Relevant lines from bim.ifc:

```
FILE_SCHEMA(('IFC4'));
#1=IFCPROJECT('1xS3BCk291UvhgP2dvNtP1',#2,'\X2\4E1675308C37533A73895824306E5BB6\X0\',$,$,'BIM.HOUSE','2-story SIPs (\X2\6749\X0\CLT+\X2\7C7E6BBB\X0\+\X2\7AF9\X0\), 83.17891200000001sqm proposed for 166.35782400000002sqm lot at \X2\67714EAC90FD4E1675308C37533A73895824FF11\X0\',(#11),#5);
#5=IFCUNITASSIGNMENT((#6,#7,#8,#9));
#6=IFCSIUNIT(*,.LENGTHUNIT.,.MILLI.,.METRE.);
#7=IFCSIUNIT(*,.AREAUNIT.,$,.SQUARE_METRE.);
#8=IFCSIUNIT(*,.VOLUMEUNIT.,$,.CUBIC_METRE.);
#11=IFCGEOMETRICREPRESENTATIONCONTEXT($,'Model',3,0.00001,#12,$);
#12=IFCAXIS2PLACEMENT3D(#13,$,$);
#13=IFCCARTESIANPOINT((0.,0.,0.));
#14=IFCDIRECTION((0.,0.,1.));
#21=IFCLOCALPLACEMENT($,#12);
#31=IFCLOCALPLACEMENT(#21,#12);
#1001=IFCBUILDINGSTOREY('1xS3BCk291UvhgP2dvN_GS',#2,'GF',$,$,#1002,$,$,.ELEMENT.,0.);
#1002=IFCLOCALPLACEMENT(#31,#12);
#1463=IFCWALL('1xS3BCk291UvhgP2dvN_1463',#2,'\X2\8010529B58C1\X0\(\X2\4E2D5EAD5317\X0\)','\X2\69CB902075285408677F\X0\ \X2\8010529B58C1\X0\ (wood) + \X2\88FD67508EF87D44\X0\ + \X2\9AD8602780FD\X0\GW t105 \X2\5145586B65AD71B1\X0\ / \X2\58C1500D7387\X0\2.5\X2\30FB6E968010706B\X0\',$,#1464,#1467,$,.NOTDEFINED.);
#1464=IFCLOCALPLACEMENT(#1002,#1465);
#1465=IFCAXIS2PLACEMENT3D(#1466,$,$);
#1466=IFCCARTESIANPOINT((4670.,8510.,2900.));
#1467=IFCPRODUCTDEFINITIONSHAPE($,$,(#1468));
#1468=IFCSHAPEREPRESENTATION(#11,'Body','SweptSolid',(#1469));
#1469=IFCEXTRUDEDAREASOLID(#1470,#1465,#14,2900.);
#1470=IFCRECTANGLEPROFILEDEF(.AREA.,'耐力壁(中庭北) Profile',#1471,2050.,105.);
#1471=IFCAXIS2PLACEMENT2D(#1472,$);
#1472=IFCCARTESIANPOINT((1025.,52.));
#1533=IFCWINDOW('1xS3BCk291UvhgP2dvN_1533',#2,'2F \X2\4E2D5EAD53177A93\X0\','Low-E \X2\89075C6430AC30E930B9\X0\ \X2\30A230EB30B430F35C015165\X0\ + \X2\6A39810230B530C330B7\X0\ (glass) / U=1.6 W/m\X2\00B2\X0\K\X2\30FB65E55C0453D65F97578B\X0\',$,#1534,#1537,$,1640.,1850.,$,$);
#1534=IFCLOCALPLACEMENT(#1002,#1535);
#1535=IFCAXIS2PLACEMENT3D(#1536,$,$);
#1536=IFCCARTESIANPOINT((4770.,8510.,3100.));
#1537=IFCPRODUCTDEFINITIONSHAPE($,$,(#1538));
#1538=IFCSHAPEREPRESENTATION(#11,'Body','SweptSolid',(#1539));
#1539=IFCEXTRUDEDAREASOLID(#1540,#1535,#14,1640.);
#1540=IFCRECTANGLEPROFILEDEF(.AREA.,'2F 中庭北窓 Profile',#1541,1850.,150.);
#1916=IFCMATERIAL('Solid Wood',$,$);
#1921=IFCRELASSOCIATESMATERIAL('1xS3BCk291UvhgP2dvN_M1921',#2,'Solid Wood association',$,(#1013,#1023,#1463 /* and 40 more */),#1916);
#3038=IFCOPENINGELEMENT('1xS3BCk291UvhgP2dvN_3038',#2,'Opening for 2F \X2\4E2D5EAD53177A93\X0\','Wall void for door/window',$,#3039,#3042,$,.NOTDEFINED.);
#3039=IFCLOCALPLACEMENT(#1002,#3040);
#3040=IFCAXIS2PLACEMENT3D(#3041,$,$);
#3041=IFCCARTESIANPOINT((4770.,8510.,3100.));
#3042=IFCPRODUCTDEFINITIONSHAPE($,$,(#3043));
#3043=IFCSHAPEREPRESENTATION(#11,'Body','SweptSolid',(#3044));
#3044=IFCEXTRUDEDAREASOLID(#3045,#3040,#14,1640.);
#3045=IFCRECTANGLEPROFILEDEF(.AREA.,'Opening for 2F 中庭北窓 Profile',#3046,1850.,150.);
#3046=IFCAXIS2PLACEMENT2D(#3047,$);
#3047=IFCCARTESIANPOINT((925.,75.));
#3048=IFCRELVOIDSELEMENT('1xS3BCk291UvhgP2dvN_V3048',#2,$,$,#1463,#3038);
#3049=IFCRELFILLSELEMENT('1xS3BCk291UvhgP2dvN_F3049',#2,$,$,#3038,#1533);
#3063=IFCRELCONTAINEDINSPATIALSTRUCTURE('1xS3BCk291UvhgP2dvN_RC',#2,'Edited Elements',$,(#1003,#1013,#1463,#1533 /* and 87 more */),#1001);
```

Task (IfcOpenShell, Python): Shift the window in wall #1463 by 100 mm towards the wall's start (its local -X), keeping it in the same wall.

```python
import ifcopenshell
import ifcopenshell.api.geometry
import ifcopenshell.util.placement

model = ifcopenshell.open("bim.ifc")

window = model.by_guid("1xS3BCk291UvhgP2dvN_1533")
opening = window.FillsVoids[0].RelatingOpeningElement
wall = opening.VoidsElements[0].RelatingBuildingElement

wall_matrix = ifcopenshell.util.placement.get_local_placement(wall.ObjectPlacement)
shift = wall_matrix[:3, 0] * -100.0
before = ifcopenshell.util.placement.get_local_placement(window.ObjectPlacement)[:3, 3].copy()

# The window is not placed relative to its opening, so move both.
for product in (opening, window):
    matrix = ifcopenshell.util.placement.get_local_placement(product.ObjectPlacement)
    matrix[:3, 3] += shift
    ifcopenshell.api.geometry.edit_object_placement(model, product=product, matrix=matrix, is_si=False)

after = ifcopenshell.util.placement.get_local_placement(window.ObjectPlacement)[:3, 3]
print("window moved by", (after - before).round(3) + 0.0)

model.write("bim_rev.ifc")
```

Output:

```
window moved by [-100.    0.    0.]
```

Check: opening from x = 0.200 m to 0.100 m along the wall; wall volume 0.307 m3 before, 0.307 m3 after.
